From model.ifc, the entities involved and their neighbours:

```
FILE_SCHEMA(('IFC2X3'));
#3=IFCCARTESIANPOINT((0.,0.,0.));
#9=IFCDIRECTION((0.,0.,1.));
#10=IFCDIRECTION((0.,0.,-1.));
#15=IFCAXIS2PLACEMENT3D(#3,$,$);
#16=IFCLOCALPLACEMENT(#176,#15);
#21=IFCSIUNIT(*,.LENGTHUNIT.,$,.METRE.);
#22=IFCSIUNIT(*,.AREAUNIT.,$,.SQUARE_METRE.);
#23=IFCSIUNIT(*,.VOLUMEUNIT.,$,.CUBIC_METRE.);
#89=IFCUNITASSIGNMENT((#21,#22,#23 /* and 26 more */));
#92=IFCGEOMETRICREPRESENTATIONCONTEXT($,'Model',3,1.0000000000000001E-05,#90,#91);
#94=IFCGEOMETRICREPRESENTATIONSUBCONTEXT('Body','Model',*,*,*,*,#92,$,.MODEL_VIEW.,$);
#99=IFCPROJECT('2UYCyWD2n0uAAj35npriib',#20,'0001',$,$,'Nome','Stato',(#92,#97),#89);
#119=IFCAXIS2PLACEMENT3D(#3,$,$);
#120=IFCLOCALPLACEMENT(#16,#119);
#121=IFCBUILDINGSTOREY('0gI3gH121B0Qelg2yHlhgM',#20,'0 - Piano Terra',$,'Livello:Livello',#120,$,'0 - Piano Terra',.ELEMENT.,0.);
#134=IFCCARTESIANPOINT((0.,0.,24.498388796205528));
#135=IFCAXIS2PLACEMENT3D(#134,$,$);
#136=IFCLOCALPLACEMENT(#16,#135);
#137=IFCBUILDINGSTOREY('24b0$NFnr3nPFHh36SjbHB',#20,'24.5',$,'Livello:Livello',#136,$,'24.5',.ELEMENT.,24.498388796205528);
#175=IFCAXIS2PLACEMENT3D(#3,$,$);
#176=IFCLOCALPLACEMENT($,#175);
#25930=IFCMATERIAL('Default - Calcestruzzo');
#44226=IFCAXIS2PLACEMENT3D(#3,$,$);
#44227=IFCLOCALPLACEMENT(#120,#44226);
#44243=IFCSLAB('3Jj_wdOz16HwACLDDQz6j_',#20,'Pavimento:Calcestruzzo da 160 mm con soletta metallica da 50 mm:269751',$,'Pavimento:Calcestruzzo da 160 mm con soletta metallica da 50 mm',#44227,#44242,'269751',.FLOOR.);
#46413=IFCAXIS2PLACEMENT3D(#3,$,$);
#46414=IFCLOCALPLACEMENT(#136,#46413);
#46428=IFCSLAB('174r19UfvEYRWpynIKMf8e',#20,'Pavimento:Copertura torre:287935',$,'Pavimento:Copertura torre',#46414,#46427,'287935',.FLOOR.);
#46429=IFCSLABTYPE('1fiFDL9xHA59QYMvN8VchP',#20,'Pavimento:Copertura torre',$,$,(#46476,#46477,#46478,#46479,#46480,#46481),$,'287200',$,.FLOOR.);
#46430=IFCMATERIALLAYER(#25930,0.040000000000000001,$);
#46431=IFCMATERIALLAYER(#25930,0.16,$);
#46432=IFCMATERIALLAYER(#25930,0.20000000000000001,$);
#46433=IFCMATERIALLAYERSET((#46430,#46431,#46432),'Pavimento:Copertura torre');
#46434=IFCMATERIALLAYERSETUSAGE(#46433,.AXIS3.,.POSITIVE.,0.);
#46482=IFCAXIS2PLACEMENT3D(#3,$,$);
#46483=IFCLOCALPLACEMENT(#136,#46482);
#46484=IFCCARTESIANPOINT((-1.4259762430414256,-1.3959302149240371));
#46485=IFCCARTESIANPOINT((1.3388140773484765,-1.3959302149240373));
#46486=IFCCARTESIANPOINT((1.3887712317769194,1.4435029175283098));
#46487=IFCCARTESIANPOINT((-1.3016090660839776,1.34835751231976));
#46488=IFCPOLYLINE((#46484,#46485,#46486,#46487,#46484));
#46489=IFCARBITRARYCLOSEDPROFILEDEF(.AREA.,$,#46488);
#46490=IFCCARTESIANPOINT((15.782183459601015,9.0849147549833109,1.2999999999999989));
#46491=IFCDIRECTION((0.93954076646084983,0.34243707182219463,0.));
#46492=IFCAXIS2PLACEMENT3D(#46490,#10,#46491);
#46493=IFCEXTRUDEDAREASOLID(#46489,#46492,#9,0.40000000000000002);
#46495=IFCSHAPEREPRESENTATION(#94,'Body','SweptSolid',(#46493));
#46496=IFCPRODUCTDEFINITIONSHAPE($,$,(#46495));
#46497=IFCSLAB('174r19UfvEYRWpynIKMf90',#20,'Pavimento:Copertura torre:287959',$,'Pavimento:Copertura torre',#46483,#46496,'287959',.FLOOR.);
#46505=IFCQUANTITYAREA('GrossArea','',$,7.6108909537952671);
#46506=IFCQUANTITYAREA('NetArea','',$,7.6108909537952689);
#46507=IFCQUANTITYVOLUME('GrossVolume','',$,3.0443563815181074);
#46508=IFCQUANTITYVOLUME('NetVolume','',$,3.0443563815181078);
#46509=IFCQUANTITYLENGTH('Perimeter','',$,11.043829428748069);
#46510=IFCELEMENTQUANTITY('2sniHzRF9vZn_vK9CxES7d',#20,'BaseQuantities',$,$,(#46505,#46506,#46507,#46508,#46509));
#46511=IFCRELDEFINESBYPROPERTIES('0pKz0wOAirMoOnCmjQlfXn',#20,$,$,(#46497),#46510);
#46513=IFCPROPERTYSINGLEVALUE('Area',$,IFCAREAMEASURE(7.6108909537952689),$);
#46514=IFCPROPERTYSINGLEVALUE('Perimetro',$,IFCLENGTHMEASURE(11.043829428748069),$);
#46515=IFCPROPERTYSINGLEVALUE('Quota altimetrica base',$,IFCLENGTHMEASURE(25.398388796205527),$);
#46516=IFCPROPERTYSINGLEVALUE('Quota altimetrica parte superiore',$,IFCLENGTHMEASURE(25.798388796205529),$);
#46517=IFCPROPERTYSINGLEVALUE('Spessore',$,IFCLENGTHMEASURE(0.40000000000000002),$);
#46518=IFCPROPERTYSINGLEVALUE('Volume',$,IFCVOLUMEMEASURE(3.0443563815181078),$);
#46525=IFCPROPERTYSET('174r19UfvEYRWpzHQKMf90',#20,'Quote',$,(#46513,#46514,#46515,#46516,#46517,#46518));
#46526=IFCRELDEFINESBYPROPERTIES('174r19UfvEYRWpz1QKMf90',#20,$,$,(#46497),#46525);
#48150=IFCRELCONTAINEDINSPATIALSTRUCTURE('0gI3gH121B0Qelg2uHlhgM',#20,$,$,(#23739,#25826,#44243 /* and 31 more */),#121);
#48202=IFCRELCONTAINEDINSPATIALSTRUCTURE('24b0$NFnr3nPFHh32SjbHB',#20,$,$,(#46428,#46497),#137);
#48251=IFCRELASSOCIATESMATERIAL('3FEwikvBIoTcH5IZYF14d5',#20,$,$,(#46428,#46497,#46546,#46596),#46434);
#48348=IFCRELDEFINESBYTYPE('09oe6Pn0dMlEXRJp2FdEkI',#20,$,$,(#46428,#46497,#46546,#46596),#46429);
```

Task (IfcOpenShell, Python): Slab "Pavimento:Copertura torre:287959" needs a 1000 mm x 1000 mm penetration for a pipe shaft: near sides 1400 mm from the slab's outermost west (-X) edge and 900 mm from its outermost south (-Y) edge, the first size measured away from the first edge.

```python
import numpy as np
import ifcopenshell
import ifcopenshell.api.feature
import ifcopenshell.api.geometry
import ifcopenshell.api.pset
import ifcopenshell.api.root
import ifcopenshell.geom
import ifcopenshell.util.element
import ifcopenshell.util.placement
import ifcopenshell.util.representation
import ifcopenshell.util.shape
import ifcopenshell.util.unit

model = ifcopenshell.open("model.ifc")
unit_scale = ifcopenshell.util.unit.calculate_unit_scale(model)
area_scale = ifcopenshell.util.unit.calculate_unit_scale(model, "AREAUNIT")
volume_scale = ifcopenshell.util.unit.calculate_unit_scale(model, "VOLUMEUNIT")
settings = ifcopenshell.geom.settings()


def volume(element):
    """Net volume in cubic metres, openings subtracted."""
    shape = ifcopenshell.geom.create_shape(settings, element)
    return ifcopenshell.util.shape.get_volume(shape.geometry)


slab = model.by_id(46497)
before = volume(slab)

# Extent in the slab's own axes, in metres. The edges named are its -X and -Y sides.
slab_shape = ifcopenshell.geom.create_shape(settings, slab)
vertices = ifcopenshell.util.shape.get_vertices(slab_shape.geometry)
x_min, y_min, bottom = vertices.min(axis=0)
top = vertices[:, 2].max()

opening = ifcopenshell.api.root.create_entity(model, ifc_class="IfcOpeningElement", name="Pipe shaft opening")
context = ifcopenshell.util.representation.get_context(model, "Model", "Body", "MODEL_VIEW")
width, depth = 1, 1
outline = [(0.0, 0.0), (width, 0.0), (width, depth), (0.0, depth), (0.0, 0.0)]
# Overshoot both faces by 50 mm so the cut is clean.
shape = ifcopenshell.api.geometry.add_slab_representation(
    model, context=context, depth=top - bottom + 0.1, polyline=outline
)
ifcopenshell.api.geometry.assign_representation(model, product=opening, representation=shape)

matrix = ifcopenshell.util.placement.get_local_placement(slab.ObjectPlacement)
matrix[:, 3] = matrix @ np.append(np.array([x_min + 1.4, y_min + 0.9, bottom - 0.05]) / unit_scale, 1.0)
ifcopenshell.api.geometry.edit_object_placement(model, product=opening, matrix=matrix, is_si=False)
ifcopenshell.api.feature.add_feature(model, feature=opening, element=slab)

after = volume(slab)

# Update the slab's stored quantities.
qto = model.by_id(ifcopenshell.util.element.get_pset(slab, "BaseQuantities", should_inherit=False)["id"])
ifcopenshell.api.pset.edit_qto(model, qto=qto, properties={
    "NetArea": after / (top - bottom) / area_scale,
    "NetVolume": after / volume_scale,
})
pset = model.by_id(ifcopenshell.util.element.get_pset(slab, "Quote", should_inherit=False)["id"])
ifcopenshell.api.pset.edit_pset(model, pset=pset, properties={
    "Area": model.create_entity("IfcAreaMeasure", after / (top - bottom) / area_scale),
    "Volume": model.create_entity("IfcVolumeMeasure", after / volume_scale),
})

print(f"slab volume {before:.3f} -> {after:.3f} m3")

model.write("model_rev.ifc")
```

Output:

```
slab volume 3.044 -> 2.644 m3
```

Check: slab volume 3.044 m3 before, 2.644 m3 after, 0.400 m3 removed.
